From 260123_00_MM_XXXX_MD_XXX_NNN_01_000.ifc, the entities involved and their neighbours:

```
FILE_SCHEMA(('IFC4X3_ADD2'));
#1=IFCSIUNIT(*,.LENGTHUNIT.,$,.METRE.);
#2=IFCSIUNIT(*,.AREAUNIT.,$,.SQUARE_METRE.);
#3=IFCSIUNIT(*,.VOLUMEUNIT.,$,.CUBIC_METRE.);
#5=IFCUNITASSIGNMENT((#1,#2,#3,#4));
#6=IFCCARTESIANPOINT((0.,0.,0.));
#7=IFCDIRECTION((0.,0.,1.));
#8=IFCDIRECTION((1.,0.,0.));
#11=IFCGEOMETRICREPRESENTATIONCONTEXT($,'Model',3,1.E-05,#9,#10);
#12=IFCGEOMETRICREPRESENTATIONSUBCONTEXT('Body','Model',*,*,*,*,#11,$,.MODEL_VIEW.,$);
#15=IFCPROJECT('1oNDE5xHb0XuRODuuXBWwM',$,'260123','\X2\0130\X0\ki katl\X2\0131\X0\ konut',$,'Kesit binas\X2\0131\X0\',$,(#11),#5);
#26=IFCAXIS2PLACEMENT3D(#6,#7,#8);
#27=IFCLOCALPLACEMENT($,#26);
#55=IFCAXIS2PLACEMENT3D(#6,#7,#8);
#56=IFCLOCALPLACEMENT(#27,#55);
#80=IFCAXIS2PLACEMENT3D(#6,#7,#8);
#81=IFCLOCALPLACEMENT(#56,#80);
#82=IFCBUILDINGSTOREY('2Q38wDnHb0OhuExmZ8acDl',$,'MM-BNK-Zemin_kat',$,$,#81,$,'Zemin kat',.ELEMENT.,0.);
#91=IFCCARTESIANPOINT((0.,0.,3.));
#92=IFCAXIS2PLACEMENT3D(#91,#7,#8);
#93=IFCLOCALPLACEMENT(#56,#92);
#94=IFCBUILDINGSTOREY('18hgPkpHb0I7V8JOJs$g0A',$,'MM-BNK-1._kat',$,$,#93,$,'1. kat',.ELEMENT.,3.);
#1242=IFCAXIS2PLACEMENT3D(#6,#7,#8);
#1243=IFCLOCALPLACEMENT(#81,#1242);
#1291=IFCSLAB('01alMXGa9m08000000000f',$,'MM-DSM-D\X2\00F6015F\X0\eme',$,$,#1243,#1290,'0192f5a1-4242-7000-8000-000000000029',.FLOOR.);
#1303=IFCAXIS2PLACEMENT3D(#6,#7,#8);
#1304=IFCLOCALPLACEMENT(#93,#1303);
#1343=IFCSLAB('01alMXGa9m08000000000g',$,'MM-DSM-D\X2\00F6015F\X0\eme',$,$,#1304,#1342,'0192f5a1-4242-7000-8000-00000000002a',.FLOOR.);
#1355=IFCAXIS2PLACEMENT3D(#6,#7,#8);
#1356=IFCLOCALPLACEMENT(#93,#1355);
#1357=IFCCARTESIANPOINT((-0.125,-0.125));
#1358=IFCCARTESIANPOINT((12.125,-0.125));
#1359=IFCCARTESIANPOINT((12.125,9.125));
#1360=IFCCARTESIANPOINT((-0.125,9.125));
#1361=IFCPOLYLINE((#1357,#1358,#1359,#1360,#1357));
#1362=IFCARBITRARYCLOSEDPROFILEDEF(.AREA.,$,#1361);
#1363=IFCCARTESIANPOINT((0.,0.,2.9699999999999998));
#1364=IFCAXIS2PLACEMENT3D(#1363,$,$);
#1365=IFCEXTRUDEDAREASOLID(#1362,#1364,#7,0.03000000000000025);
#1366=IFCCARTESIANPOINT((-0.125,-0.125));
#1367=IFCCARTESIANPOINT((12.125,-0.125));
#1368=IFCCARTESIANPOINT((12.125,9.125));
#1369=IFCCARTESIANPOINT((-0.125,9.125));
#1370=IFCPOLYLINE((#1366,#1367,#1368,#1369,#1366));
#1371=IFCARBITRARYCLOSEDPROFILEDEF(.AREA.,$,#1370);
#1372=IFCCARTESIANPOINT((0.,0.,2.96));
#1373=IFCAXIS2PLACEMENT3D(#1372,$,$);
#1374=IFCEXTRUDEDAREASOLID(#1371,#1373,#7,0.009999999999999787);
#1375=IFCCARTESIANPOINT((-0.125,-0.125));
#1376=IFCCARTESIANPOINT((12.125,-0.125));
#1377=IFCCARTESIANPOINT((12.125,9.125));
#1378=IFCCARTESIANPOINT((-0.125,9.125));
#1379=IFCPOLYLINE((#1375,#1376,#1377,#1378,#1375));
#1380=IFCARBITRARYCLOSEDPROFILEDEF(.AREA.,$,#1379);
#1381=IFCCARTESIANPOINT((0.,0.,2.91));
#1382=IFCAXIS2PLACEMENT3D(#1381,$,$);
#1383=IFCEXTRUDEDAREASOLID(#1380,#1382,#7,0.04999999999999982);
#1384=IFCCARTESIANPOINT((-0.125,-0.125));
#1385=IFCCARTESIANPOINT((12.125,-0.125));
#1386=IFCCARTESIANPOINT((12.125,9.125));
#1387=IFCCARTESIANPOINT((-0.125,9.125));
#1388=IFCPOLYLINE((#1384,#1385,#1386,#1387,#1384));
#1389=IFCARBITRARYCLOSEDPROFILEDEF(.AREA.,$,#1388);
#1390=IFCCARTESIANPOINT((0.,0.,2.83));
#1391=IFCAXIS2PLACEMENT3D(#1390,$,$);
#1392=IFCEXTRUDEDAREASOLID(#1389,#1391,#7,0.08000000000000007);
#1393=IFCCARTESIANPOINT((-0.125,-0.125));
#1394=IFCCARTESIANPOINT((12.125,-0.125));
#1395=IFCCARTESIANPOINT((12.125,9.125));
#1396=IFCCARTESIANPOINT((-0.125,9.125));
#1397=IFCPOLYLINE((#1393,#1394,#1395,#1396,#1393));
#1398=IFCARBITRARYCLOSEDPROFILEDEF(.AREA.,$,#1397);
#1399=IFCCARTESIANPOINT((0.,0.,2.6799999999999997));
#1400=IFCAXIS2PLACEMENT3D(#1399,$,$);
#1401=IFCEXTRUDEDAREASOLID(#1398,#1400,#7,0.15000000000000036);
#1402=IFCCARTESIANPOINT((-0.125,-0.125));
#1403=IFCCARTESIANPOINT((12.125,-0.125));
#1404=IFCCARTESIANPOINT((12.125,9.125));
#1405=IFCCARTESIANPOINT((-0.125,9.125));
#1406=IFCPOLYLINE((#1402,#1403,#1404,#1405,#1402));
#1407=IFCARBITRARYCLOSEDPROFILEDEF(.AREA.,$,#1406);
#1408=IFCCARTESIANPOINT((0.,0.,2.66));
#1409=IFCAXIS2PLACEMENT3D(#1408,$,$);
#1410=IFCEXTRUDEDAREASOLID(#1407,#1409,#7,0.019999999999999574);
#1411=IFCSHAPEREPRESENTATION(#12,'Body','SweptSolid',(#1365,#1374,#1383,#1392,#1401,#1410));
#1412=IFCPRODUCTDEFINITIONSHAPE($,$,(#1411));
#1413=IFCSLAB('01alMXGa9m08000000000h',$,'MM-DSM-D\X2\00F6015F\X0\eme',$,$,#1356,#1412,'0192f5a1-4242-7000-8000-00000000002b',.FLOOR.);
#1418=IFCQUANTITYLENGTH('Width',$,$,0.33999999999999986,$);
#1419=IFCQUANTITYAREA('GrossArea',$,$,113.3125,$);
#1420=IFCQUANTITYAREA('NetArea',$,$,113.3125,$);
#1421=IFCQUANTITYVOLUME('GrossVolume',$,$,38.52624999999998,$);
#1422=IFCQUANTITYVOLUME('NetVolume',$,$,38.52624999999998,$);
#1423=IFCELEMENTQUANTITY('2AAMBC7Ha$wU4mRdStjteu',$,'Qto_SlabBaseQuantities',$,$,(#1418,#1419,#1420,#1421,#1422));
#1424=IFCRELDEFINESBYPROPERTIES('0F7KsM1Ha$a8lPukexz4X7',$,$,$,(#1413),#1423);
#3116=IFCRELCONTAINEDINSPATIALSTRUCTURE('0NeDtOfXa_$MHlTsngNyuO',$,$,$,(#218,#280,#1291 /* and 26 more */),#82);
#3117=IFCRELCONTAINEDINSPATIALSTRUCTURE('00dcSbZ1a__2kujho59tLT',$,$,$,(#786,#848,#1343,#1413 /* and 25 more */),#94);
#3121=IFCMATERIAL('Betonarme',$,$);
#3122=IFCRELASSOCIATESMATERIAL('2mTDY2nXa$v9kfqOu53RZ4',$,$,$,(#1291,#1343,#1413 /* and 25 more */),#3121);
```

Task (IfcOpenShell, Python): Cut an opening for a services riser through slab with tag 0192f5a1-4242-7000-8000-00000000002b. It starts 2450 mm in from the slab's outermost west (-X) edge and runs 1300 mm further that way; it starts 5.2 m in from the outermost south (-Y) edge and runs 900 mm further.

```python
import numpy as np
import ifcopenshell
import ifcopenshell.api.feature
import ifcopenshell.api.geometry
import ifcopenshell.api.pset
import ifcopenshell.api.root
import ifcopenshell.geom
import ifcopenshell.util.element
import ifcopenshell.util.placement
import ifcopenshell.util.representation
import ifcopenshell.util.shape
import ifcopenshell.util.unit

model = ifcopenshell.open("260123_00_MM_XXXX_MD_XXX_NNN_01_000.ifc")
unit_scale = ifcopenshell.util.unit.calculate_unit_scale(model)
area_scale = ifcopenshell.util.unit.calculate_unit_scale(model, "AREAUNIT")
volume_scale = ifcopenshell.util.unit.calculate_unit_scale(model, "VOLUMEUNIT")
settings = ifcopenshell.geom.settings()


def volume(element):
    """Net volume in cubic metres, openings subtracted."""
    shape = ifcopenshell.geom.create_shape(settings, element)
    return ifcopenshell.util.shape.get_volume(shape.geometry)


slab = model.by_guid("01alMXGa9m08000000000h")
before = volume(slab)

# Extent in the slab's own axes, in metres. The edges named are its -X and -Y sides.
slab_shape = ifcopenshell.geom.create_shape(settings, slab)
vertices = ifcopenshell.util.shape.get_vertices(slab_shape.geometry)
x_min, y_min, bottom = vertices.min(axis=0)
top = vertices[:, 2].max()

opening = ifcopenshell.api.root.create_entity(model, ifc_class="IfcOpeningElement", name="Services riser opening", predefined_type="OPENING")
context = ifcopenshell.util.representation.get_context(model, "Model", "Body", "MODEL_VIEW")
width, depth = 1.3, 0.9
outline = [(0.0, 0.0), (width, 0.0), (width, depth), (0.0, depth), (0.0, 0.0)]
# Overshoot both faces by 50 mm so the cut is clean.
shape = ifcopenshell.api.geometry.add_slab_representation(
    model, context=context, depth=top - bottom + 0.1, polyline=outline
)
ifcopenshell.api.geometry.assign_representation(model, product=opening, representation=shape)

matrix = ifcopenshell.util.placement.get_local_placement(slab.ObjectPlacement)
matrix[:, 3] = matrix @ np.append(np.array([x_min + 2.45, y_min + 5.2, bottom - 0.05]) / unit_scale, 1.0)
ifcopenshell.api.geometry.edit_object_placement(model, product=opening, matrix=matrix, is_si=False)
ifcopenshell.api.feature.add_feature(model, feature=opening, element=slab)

after = volume(slab)

# Update the slab's stored quantities.
qto = model.by_id(ifcopenshell.util.element.get_pset(slab, "Qto_SlabBaseQuantities", should_inherit=False)["id"])
ifcopenshell.api.pset.edit_qto(model, qto=qto, properties={
    "NetArea": after / (top - bottom) / area_scale,
    "NetVolume": after / volume_scale,
})

print(f"slab volume {before:.3f} -> {after:.3f} m3")

model.write("260123_00_MM_XXXX_MD_XXX_NNN_01_000_v2.ifc")
```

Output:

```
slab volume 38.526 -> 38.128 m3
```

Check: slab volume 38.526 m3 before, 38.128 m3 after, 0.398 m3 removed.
